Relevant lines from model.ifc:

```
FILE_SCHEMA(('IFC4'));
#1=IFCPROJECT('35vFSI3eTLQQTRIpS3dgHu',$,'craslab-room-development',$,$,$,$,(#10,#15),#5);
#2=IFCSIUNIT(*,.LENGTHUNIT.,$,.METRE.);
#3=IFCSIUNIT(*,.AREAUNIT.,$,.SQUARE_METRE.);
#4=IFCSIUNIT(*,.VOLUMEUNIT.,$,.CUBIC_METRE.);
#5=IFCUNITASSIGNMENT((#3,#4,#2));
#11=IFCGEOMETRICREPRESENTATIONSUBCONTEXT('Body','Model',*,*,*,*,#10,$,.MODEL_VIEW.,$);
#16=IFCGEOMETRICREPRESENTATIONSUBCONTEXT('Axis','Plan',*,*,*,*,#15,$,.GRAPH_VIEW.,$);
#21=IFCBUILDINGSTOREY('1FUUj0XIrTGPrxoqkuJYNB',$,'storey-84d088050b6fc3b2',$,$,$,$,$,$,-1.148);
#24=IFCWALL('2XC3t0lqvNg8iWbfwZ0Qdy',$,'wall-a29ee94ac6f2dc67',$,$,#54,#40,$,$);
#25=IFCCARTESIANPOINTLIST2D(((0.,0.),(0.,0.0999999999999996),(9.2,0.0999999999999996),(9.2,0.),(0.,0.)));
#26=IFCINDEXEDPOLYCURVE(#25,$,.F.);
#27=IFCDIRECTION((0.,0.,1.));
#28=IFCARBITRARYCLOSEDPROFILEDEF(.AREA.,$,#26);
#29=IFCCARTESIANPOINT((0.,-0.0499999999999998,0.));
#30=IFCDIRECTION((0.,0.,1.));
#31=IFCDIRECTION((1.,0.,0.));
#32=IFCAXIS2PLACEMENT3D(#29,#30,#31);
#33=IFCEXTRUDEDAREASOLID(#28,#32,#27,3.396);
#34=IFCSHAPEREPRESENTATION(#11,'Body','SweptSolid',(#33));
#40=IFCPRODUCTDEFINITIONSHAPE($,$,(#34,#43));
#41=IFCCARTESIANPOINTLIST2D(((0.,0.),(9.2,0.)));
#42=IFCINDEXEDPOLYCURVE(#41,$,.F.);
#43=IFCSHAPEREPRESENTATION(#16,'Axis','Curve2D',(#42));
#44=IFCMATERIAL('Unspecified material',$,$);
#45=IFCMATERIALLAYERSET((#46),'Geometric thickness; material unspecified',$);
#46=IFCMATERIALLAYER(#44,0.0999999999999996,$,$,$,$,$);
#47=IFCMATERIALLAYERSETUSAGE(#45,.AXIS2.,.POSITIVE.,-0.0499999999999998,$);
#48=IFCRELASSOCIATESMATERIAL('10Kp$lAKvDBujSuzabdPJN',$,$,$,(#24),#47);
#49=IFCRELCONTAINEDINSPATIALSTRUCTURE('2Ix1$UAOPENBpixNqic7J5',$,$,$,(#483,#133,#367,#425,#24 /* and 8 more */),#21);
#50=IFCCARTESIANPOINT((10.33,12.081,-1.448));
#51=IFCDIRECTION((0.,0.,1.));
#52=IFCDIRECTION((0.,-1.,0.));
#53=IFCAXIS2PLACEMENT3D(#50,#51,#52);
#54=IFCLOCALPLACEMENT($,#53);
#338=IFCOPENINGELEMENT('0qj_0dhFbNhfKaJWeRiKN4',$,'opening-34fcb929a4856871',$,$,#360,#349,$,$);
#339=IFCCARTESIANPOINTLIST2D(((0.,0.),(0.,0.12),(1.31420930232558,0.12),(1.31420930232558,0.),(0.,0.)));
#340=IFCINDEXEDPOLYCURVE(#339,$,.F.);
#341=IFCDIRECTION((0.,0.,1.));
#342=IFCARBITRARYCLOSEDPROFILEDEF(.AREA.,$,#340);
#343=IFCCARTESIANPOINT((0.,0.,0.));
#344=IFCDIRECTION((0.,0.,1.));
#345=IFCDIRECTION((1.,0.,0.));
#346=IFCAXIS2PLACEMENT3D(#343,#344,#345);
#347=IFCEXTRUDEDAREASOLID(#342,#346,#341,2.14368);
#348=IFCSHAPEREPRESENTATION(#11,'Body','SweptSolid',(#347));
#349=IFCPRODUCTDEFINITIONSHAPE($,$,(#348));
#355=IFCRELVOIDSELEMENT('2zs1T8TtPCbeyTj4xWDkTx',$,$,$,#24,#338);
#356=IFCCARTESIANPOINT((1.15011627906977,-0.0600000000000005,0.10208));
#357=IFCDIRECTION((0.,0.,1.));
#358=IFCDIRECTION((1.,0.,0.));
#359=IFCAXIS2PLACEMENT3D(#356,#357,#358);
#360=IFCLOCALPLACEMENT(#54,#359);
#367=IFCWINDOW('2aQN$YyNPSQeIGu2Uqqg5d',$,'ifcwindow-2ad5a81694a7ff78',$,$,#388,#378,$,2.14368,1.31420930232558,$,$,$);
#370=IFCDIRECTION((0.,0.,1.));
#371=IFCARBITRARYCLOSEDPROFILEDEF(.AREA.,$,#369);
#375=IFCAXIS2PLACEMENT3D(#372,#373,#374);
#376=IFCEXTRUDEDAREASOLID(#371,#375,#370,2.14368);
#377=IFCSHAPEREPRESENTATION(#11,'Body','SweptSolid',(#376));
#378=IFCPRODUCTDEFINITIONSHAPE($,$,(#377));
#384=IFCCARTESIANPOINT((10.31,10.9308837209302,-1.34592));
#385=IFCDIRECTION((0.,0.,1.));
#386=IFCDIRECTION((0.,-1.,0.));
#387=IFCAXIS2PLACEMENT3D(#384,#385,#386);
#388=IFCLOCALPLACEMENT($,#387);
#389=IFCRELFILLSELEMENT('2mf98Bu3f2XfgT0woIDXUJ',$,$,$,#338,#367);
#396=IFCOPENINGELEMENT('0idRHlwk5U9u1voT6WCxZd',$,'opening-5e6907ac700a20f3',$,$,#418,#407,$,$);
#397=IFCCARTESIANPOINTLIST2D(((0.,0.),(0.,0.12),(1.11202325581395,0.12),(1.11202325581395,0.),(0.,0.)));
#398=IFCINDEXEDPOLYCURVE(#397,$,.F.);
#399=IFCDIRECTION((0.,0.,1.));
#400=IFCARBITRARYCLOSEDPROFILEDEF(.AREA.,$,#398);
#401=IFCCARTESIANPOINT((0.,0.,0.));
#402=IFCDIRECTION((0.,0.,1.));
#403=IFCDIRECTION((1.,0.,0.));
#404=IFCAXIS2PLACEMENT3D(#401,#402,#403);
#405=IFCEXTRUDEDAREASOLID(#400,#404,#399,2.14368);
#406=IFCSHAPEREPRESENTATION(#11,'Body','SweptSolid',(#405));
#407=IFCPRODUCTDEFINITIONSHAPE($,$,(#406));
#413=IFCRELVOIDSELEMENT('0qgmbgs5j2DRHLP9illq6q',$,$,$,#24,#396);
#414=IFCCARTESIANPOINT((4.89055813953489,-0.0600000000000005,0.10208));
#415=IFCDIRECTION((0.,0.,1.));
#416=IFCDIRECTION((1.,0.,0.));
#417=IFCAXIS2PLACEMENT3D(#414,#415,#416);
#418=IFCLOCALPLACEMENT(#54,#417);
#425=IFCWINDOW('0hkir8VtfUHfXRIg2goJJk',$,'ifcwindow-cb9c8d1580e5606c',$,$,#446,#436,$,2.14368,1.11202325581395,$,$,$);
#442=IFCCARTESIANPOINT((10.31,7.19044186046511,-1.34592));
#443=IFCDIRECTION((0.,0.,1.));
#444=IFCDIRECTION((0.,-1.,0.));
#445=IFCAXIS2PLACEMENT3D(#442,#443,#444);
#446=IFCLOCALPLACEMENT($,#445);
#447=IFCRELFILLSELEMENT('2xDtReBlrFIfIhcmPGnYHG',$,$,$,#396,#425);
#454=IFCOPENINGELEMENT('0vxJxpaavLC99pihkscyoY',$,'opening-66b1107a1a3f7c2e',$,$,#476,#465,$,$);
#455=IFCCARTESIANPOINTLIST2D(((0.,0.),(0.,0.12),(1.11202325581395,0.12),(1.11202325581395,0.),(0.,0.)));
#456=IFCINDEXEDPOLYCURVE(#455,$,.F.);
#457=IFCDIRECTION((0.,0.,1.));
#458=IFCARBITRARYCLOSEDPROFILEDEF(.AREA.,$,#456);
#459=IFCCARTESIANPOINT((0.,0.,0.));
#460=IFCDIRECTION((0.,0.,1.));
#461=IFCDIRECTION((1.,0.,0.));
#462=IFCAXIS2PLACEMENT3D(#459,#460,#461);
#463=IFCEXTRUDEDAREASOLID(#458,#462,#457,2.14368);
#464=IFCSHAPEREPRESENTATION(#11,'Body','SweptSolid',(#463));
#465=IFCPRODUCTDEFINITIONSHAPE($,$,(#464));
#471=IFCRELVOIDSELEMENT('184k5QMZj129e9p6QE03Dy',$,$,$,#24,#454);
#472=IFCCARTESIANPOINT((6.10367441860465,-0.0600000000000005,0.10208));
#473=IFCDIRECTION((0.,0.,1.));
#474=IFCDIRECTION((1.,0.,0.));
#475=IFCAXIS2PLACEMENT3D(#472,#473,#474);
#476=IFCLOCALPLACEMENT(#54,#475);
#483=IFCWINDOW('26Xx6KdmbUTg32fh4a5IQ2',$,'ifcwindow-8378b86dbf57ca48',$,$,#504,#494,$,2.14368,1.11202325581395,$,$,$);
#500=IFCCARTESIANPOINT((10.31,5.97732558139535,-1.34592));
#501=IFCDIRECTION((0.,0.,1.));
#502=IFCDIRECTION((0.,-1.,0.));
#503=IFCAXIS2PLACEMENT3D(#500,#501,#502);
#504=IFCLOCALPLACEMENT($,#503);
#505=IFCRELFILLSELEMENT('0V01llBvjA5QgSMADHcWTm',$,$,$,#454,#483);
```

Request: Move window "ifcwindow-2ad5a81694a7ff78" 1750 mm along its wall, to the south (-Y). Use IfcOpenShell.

```python
import ifcopenshell
import ifcopenshell.api.geometry
import ifcopenshell.util.placement
import ifcopenshell.util.unit

model = ifcopenshell.open("model.ifc")
unit_scale = ifcopenshell.util.unit.calculate_unit_scale(model)

window = model.by_guid("2aQN$YyNPSQeIGu2Uqqg5d")
opening = window.FillsVoids[0].RelatingOpeningElement
wall = opening.VoidsElements[0].RelatingBuildingElement

wall_matrix = ifcopenshell.util.placement.get_local_placement(wall.ObjectPlacement)
shift = wall_matrix[:3, 0] * 1.75 / unit_scale
before = ifcopenshell.util.placement.get_local_placement(window.ObjectPlacement)[:3, 3].copy()

# The window is not placed relative to its opening, so move both.
for product in (opening, window):
    matrix = ifcopenshell.util.placement.get_local_placement(product.ObjectPlacement)
    matrix[:3, 3] += shift
    ifcopenshell.api.geometry.edit_object_placement(model, product=product, matrix=matrix, is_si=False)

after = ifcopenshell.util.placement.get_local_placement(window.ObjectPlacement)[:3, 3]
print("window moved by", (after - before).round(3) + 0.0)

model.write("model_edited.ifc")
```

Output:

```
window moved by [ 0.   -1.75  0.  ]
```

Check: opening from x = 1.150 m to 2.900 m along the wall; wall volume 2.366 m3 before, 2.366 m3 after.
